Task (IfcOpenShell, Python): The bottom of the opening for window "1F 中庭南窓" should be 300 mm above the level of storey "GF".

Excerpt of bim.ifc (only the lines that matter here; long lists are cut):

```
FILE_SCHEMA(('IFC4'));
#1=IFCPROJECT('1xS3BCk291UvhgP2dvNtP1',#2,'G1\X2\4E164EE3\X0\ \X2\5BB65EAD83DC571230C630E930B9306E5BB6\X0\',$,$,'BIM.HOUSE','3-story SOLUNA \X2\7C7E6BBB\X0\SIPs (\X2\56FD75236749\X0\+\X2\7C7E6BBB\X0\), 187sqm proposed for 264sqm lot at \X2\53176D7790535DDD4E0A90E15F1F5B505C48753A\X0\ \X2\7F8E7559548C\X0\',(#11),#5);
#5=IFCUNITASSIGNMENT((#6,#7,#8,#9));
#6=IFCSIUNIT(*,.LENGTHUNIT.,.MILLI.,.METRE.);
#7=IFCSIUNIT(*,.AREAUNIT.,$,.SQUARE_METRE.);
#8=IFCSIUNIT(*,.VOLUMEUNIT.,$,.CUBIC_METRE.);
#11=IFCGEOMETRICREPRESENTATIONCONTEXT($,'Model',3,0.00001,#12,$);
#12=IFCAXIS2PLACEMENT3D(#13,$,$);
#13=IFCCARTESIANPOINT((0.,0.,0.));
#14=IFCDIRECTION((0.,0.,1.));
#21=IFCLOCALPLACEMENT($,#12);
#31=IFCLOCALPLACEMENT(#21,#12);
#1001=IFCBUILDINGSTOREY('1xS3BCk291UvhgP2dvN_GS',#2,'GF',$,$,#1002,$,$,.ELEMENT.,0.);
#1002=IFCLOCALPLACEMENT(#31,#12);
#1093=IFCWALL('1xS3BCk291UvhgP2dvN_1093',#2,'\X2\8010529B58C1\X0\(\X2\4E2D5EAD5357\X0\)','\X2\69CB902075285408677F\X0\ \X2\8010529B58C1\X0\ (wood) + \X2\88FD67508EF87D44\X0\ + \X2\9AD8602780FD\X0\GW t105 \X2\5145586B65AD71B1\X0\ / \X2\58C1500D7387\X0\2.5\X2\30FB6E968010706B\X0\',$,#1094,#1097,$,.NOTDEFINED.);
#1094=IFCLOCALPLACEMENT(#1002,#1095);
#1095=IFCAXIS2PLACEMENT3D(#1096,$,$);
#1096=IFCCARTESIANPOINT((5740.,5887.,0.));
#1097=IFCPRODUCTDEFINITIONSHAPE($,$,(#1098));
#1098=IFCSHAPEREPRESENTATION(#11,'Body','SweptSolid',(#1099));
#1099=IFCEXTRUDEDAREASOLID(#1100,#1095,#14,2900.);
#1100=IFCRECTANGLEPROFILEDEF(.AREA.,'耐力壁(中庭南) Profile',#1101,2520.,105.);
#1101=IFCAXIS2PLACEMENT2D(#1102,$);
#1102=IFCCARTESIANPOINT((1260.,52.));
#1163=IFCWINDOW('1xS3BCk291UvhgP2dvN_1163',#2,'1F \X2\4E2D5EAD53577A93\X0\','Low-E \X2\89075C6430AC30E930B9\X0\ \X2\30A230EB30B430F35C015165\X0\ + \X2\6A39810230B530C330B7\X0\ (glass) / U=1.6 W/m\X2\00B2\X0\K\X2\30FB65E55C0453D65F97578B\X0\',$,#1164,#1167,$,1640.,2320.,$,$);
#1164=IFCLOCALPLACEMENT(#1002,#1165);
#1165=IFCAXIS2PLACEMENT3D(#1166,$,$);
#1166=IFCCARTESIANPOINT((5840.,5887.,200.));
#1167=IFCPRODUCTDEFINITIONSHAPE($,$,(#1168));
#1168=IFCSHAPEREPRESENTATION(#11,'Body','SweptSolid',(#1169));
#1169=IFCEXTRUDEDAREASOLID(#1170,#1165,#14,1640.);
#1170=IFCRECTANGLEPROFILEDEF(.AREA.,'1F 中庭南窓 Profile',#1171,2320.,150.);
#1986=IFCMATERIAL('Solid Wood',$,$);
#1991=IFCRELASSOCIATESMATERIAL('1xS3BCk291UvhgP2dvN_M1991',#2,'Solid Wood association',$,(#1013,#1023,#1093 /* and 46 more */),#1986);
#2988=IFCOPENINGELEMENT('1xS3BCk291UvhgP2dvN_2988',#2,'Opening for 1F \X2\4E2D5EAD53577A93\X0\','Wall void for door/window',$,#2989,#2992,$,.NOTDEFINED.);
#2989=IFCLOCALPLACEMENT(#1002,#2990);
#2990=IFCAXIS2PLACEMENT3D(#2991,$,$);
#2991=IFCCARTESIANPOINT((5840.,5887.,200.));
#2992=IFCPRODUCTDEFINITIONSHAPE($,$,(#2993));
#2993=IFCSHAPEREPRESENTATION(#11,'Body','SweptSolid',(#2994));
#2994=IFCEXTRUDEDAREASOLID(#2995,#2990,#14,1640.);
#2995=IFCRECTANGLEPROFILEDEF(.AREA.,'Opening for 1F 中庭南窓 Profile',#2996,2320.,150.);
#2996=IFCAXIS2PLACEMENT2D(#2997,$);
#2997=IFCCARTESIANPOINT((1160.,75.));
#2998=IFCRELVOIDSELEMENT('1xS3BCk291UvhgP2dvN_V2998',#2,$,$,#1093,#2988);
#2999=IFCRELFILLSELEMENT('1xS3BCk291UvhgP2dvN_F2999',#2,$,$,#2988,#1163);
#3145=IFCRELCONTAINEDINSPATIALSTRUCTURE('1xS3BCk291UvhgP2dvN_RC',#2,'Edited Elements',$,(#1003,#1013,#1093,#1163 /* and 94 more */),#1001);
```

```python
import numpy as np
import ifcopenshell
import ifcopenshell.api.geometry
import ifcopenshell.geom
import ifcopenshell.util.element
import ifcopenshell.util.placement
import ifcopenshell.util.shape
import ifcopenshell.util.unit

model = ifcopenshell.open("bim.ifc")
unit_scale = ifcopenshell.util.unit.calculate_unit_scale(model)

window = model.by_guid("1xS3BCk291UvhgP2dvN_1163")
opening = window.FillsVoids[0].RelatingOpeningElement
storey = ifcopenshell.util.element.get_container(window, ifc_class="IfcBuildingStorey")
level = ifcopenshell.util.placement.get_local_placement(storey.ObjectPlacement)[2, 3]

# The opening's origin need not be at the sill, so measure its lowest point.
shape = ifcopenshell.geom.create_shape(ifcopenshell.geom.settings(), opening)
bottom = ifcopenshell.util.shape.get_shape_bottom_elevation(shape, shape.geometry) / unit_scale
dz = level + 0.3 / unit_scale - bottom

shift = np.array([0.0, 0.0, dz])
# The window is not placed relative to its opening, so move both.
for product in (opening, window):
    matrix = ifcopenshell.util.placement.get_local_placement(product.ObjectPlacement)
    matrix[:3, 3] += shift
    ifcopenshell.api.geometry.edit_object_placement(model, product=product, matrix=matrix, is_si=False)

print(f"moved by {dz * unit_scale:+.3f} m")

model.write("bim_updated.ifc")
```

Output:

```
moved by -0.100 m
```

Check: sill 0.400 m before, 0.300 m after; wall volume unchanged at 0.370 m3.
